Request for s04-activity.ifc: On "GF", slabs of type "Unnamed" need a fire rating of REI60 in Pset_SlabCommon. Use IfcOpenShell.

First a look at what the model holds.

```python
import ifcopenshell
import ifcopenshell.util.element

model = ifcopenshell.open("s04-activity.ifc")
print(model.schema)
storey = next(s for s in model.by_type("IfcBuildingStorey") if s.Name == "GF")
slabs = [e for e in ifcopenshell.util.element.get_decomposition(storey) if e.is_a("IfcSlab")]
seen = {}
for e in slabs:
    element_type = ifcopenshell.util.element.get_type(e)
    key = (element_type.Name if element_type != e and element_type else None, ifcopenshell.util.element.get_pset(e, "Pset_SlabCommon", "FireRating"))
    seen[key] = seen.get(key, 0) + 1
for (name, value), count in sorted(seen.items(), key=str):
    print(count, "x", name, "|", value)
```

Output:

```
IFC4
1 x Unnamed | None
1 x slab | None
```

```python
import ifcopenshell
import ifcopenshell.api.pset
import ifcopenshell.util.element

model = ifcopenshell.open("s04-activity.ifc")

storey = next(s for s in model.by_type("IfcBuildingStorey") if s.Name == "GF")
slabs = [e for e in ifcopenshell.util.element.get_decomposition(storey) if e.is_a("IfcSlab")]

count = 0
for e in slabs:
    element_type = ifcopenshell.util.element.get_type(e)
    if element_type in (None, e) or element_type.Name != "Unnamed":
        continue
    # add_pset returns the element's existing set when there is one.
    pset = ifcopenshell.api.pset.add_pset(model, product=e, name="Pset_SlabCommon")
    ifcopenshell.api.pset.edit_pset(model, pset=pset, properties={"FireRating": "REI60"})
    count += 1

print(count, "slabs updated")

model.write("s04-activity_edited.ifc")
```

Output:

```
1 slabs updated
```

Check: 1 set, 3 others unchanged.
